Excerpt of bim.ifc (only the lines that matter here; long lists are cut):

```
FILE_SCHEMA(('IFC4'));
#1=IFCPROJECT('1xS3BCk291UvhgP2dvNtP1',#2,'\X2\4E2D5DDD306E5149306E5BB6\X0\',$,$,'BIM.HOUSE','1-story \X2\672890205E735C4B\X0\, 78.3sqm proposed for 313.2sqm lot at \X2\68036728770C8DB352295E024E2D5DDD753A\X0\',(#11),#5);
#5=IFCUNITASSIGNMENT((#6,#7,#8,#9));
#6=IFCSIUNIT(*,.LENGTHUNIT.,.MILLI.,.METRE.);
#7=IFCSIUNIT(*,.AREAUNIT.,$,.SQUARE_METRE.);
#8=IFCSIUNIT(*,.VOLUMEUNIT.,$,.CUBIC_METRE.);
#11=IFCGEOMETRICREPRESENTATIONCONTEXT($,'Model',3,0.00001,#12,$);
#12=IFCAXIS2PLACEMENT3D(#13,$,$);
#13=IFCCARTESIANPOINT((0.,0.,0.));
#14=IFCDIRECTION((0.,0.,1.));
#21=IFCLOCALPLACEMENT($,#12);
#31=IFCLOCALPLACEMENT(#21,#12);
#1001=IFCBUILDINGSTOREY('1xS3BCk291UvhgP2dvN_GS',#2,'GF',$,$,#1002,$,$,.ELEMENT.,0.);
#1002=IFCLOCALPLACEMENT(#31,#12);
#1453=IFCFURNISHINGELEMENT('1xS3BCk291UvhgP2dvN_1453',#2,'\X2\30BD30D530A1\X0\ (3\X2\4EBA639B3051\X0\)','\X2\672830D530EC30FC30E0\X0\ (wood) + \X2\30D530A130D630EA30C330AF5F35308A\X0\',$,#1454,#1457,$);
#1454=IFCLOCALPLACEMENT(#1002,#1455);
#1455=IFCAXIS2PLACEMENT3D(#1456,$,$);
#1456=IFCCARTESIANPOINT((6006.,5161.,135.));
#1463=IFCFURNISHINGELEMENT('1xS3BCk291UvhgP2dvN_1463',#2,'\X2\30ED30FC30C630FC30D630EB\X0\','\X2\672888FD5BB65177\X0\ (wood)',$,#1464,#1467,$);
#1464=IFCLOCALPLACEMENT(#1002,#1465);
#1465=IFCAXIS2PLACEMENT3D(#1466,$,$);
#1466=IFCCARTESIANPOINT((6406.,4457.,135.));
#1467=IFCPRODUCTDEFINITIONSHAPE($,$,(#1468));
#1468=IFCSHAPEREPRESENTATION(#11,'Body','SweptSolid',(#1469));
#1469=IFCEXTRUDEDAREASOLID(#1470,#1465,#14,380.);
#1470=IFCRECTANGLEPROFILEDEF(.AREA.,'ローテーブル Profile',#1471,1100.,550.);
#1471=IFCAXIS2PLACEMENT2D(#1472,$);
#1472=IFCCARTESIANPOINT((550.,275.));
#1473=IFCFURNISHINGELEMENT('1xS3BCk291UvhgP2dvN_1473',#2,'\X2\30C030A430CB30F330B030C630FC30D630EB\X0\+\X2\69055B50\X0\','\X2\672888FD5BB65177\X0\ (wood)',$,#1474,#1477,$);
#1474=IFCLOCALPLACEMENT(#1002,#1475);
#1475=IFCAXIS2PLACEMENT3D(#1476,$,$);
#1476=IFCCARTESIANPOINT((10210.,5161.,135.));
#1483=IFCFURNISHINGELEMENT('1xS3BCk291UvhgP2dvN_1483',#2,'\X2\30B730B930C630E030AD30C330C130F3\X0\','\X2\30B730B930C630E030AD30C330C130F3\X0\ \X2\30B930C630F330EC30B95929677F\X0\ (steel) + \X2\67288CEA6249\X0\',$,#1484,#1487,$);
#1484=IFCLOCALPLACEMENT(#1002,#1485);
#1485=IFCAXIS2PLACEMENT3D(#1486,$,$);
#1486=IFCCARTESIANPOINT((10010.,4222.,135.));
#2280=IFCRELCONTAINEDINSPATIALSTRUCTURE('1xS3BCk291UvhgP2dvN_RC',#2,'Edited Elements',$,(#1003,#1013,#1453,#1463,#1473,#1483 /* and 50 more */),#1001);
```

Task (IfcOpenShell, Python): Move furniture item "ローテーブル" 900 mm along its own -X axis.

```python
import ifcopenshell
import ifcopenshell.api.geometry
import ifcopenshell.util.placement
import ifcopenshell.util.unit

model = ifcopenshell.open("bim.ifc")
unit_scale = ifcopenshell.util.unit.calculate_unit_scale(model)

item = model.by_guid("1xS3BCk291UvhgP2dvN_1463")
matrix = ifcopenshell.util.placement.get_local_placement(item.ObjectPlacement)
matrix[:3, 3] -= matrix[:3, 0] * 0.9 / unit_scale
ifcopenshell.api.geometry.edit_object_placement(model, product=item, matrix=matrix, is_si=False)

print(ifcopenshell.util.placement.get_local_placement(item.ObjectPlacement).round(3) + 0.0)

model.write("bim-out.ifc")
```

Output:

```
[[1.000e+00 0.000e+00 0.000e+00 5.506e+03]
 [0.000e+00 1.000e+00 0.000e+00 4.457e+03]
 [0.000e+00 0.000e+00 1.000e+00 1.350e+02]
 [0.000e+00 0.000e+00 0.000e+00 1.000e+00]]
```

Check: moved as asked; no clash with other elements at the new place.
